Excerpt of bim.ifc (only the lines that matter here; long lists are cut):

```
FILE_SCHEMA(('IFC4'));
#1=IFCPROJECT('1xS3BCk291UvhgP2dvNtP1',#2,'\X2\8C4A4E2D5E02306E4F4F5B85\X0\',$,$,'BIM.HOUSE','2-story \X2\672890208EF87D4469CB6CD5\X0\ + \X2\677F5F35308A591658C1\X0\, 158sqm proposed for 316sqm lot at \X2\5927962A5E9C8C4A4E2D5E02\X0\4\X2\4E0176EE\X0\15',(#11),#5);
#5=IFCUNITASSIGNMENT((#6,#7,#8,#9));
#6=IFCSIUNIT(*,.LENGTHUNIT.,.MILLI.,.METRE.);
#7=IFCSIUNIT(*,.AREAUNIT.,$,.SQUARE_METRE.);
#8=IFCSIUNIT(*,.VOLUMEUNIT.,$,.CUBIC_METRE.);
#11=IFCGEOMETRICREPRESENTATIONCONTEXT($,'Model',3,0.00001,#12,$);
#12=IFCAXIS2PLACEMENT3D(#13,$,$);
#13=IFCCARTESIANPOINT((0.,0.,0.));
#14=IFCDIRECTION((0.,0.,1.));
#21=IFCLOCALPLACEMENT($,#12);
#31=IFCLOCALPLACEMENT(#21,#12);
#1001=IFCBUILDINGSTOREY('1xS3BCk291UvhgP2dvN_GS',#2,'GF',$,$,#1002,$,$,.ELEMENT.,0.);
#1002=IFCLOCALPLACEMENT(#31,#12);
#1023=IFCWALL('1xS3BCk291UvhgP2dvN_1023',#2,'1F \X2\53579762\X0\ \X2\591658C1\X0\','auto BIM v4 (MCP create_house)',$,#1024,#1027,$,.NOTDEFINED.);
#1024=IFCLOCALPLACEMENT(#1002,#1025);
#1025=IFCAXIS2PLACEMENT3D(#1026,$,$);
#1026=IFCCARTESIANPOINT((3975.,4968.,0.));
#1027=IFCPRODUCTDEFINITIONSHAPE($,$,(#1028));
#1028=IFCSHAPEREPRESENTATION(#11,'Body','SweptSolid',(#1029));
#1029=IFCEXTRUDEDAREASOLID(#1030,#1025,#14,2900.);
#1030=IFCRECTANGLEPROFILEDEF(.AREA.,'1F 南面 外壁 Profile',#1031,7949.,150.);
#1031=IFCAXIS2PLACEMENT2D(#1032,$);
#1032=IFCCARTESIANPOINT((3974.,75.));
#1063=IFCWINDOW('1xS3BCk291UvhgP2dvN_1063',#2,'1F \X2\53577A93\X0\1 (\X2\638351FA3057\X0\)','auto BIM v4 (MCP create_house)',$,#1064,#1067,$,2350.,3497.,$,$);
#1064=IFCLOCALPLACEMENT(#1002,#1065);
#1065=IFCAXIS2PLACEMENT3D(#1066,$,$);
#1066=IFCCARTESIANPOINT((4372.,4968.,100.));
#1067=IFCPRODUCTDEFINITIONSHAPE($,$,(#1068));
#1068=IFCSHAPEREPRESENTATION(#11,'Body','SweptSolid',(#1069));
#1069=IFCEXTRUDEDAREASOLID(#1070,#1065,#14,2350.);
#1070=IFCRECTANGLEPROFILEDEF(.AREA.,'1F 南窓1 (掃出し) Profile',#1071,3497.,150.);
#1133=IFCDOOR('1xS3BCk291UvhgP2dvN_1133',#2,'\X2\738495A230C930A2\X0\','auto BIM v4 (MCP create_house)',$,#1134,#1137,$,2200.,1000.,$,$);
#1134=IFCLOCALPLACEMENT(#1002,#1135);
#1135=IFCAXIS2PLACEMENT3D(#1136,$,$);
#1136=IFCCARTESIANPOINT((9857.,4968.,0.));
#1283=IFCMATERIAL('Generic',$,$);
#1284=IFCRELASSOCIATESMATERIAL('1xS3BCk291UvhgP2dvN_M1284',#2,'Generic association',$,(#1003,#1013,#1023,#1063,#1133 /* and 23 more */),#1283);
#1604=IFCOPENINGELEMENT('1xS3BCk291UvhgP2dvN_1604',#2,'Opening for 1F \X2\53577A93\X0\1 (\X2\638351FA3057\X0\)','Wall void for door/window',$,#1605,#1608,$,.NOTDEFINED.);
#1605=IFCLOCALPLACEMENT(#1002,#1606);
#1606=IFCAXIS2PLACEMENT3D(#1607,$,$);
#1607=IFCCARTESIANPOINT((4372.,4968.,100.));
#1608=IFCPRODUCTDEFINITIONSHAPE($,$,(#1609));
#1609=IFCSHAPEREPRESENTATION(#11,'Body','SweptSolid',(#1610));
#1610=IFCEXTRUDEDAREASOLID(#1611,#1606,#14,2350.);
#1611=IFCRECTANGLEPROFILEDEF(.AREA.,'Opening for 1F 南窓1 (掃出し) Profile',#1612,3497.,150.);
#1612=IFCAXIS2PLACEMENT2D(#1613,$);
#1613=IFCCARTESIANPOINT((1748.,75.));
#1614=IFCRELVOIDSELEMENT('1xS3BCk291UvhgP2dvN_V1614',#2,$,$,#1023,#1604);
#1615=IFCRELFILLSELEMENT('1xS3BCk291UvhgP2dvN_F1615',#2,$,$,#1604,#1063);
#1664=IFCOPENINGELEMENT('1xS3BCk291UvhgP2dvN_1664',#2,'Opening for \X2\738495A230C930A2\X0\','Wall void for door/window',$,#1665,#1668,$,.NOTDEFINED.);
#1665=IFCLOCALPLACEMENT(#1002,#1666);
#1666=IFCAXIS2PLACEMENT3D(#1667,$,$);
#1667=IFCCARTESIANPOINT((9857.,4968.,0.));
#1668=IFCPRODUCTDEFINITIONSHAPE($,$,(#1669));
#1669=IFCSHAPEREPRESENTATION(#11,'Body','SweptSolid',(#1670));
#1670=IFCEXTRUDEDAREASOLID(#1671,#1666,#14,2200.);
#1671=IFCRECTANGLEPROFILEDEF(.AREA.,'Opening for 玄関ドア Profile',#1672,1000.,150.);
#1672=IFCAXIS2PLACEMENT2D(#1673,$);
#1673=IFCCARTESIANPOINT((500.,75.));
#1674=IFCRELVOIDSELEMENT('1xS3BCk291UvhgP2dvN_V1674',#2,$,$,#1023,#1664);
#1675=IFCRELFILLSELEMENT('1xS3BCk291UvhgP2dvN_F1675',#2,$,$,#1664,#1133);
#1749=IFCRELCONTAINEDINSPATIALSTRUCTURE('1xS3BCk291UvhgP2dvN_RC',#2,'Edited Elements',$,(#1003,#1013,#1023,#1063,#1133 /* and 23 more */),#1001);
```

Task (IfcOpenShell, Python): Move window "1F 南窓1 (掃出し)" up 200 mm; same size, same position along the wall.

```python
import numpy as np
import ifcopenshell
import ifcopenshell.api.geometry
import ifcopenshell.util.placement
import ifcopenshell.util.unit

model = ifcopenshell.open("bim.ifc")
unit_scale = ifcopenshell.util.unit.calculate_unit_scale(model)

window = model.by_guid("1xS3BCk291UvhgP2dvN_1063")
opening = window.FillsVoids[0].RelatingOpeningElement
dz = 0.2 / unit_scale

shift = np.array([0.0, 0.0, dz])
# The window is not placed relative to its opening, so move both.
for product in (opening, window):
    matrix = ifcopenshell.util.placement.get_local_placement(product.ObjectPlacement)
    matrix[:3, 3] += shift
    ifcopenshell.api.geometry.edit_object_placement(model, product=product, matrix=matrix, is_si=False)

print(f"moved by {dz * unit_scale:+.3f} m")

model.write("bim_rev.ifc")
```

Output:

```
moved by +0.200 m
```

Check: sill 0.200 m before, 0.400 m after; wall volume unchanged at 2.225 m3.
